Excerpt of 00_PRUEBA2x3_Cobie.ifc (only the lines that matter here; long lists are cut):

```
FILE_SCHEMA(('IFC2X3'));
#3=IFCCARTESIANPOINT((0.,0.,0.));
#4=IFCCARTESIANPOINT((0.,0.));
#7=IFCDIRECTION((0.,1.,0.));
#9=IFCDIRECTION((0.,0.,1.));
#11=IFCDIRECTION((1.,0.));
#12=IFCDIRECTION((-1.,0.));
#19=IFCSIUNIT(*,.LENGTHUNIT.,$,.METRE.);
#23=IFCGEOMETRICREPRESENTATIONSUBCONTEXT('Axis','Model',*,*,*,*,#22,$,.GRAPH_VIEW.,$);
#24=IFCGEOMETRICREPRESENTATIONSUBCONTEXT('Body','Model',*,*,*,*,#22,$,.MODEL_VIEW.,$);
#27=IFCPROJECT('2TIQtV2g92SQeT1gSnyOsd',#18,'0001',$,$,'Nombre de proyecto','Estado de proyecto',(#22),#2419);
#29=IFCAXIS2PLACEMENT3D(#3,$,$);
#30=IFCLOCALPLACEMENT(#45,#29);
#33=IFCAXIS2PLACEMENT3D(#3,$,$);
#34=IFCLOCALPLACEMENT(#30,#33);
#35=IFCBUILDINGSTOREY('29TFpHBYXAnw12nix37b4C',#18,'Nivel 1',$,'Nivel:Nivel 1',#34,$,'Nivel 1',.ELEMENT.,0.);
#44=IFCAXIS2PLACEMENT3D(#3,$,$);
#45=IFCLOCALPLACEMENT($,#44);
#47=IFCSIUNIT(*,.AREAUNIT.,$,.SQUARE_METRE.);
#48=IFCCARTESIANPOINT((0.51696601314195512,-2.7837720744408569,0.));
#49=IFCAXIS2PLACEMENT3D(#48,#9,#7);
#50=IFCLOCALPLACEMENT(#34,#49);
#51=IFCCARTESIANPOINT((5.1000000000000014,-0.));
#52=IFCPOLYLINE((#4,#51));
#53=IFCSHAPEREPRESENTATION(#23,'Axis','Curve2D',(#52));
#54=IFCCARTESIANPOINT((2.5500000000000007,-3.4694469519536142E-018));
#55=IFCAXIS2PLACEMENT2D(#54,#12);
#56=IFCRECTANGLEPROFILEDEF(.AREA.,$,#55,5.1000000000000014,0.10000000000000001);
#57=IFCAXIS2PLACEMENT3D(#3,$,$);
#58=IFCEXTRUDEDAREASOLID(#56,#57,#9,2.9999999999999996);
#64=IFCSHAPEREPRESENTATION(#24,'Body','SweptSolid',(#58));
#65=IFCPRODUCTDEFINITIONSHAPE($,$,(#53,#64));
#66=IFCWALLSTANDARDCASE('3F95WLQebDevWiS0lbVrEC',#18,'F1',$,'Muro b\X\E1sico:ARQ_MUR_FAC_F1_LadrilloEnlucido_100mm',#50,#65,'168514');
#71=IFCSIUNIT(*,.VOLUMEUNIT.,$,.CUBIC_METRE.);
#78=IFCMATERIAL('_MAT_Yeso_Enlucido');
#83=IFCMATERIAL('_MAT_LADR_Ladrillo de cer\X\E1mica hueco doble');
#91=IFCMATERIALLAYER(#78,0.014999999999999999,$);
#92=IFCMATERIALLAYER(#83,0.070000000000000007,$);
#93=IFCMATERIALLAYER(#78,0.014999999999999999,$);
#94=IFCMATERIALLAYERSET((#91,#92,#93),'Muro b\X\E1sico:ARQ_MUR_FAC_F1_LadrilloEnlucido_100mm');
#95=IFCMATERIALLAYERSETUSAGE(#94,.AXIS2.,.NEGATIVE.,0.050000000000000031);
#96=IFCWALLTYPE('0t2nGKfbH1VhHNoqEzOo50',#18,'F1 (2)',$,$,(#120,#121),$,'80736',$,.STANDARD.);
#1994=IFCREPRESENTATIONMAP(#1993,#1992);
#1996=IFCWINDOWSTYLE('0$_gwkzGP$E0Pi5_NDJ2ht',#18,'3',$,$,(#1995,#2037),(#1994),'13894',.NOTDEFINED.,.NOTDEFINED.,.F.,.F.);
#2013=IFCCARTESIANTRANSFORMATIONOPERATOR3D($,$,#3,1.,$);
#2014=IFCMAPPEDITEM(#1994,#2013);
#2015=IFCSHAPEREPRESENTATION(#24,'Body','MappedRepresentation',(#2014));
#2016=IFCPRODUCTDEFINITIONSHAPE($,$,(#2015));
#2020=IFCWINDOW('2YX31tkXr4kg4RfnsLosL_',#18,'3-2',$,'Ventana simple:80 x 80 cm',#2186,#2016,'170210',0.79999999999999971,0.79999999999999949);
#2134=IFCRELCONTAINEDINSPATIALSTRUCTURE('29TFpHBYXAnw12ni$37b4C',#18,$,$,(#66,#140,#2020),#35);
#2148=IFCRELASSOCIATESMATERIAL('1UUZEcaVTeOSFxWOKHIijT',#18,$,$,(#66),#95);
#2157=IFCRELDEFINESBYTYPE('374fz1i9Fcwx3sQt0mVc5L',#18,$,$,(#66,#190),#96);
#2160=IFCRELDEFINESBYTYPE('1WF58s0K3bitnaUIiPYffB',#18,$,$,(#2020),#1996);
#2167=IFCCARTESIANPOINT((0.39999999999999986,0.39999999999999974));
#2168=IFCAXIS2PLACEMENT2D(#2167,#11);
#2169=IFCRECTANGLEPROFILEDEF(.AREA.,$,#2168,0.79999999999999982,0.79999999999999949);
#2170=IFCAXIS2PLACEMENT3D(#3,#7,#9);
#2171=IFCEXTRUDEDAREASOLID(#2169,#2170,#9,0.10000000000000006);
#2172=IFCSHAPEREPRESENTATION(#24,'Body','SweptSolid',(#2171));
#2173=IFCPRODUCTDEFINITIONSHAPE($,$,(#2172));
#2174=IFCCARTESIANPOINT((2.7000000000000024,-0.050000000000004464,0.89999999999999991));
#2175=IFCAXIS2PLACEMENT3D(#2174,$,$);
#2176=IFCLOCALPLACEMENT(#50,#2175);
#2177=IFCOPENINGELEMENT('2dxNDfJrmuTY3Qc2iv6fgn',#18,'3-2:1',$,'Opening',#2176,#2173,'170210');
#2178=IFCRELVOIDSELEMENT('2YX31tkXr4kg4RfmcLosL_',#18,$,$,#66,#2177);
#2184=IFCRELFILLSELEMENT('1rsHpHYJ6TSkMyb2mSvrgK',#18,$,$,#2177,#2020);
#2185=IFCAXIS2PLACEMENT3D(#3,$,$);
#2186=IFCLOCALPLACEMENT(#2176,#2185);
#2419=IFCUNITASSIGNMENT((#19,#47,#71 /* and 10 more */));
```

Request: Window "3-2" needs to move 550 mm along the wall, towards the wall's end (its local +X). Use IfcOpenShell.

```python
import ifcopenshell
import ifcopenshell.api.geometry
import ifcopenshell.util.placement
import ifcopenshell.util.unit

model = ifcopenshell.open("00_PRUEBA2x3_Cobie.ifc")
unit_scale = ifcopenshell.util.unit.calculate_unit_scale(model)

window = model.by_guid("2YX31tkXr4kg4RfnsLosL_")
opening = window.FillsVoids[0].RelatingOpeningElement
wall = opening.VoidsElements[0].RelatingBuildingElement

wall_matrix = ifcopenshell.util.placement.get_local_placement(wall.ObjectPlacement)
shift = wall_matrix[:3, 0] * 0.55 / unit_scale
before = ifcopenshell.util.placement.get_local_placement(window.ObjectPlacement)[:3, 3].copy()

# The window is placed relative to its opening, so it follows when the opening moves.
matrix = ifcopenshell.util.placement.get_local_placement(opening.ObjectPlacement)
matrix[:3, 3] += shift
ifcopenshell.api.geometry.edit_object_placement(
    model, product=opening, matrix=matrix, is_si=False, should_transform_children=True
)

after = ifcopenshell.util.placement.get_local_placement(window.ObjectPlacement)[:3, 3]
print("window moved by", (after - before).round(3) + 0.0)

model.write("00_PRUEBA2x3_Cobie-out.ifc")
```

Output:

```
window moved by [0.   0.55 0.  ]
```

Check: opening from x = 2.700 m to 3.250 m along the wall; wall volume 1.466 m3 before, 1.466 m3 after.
